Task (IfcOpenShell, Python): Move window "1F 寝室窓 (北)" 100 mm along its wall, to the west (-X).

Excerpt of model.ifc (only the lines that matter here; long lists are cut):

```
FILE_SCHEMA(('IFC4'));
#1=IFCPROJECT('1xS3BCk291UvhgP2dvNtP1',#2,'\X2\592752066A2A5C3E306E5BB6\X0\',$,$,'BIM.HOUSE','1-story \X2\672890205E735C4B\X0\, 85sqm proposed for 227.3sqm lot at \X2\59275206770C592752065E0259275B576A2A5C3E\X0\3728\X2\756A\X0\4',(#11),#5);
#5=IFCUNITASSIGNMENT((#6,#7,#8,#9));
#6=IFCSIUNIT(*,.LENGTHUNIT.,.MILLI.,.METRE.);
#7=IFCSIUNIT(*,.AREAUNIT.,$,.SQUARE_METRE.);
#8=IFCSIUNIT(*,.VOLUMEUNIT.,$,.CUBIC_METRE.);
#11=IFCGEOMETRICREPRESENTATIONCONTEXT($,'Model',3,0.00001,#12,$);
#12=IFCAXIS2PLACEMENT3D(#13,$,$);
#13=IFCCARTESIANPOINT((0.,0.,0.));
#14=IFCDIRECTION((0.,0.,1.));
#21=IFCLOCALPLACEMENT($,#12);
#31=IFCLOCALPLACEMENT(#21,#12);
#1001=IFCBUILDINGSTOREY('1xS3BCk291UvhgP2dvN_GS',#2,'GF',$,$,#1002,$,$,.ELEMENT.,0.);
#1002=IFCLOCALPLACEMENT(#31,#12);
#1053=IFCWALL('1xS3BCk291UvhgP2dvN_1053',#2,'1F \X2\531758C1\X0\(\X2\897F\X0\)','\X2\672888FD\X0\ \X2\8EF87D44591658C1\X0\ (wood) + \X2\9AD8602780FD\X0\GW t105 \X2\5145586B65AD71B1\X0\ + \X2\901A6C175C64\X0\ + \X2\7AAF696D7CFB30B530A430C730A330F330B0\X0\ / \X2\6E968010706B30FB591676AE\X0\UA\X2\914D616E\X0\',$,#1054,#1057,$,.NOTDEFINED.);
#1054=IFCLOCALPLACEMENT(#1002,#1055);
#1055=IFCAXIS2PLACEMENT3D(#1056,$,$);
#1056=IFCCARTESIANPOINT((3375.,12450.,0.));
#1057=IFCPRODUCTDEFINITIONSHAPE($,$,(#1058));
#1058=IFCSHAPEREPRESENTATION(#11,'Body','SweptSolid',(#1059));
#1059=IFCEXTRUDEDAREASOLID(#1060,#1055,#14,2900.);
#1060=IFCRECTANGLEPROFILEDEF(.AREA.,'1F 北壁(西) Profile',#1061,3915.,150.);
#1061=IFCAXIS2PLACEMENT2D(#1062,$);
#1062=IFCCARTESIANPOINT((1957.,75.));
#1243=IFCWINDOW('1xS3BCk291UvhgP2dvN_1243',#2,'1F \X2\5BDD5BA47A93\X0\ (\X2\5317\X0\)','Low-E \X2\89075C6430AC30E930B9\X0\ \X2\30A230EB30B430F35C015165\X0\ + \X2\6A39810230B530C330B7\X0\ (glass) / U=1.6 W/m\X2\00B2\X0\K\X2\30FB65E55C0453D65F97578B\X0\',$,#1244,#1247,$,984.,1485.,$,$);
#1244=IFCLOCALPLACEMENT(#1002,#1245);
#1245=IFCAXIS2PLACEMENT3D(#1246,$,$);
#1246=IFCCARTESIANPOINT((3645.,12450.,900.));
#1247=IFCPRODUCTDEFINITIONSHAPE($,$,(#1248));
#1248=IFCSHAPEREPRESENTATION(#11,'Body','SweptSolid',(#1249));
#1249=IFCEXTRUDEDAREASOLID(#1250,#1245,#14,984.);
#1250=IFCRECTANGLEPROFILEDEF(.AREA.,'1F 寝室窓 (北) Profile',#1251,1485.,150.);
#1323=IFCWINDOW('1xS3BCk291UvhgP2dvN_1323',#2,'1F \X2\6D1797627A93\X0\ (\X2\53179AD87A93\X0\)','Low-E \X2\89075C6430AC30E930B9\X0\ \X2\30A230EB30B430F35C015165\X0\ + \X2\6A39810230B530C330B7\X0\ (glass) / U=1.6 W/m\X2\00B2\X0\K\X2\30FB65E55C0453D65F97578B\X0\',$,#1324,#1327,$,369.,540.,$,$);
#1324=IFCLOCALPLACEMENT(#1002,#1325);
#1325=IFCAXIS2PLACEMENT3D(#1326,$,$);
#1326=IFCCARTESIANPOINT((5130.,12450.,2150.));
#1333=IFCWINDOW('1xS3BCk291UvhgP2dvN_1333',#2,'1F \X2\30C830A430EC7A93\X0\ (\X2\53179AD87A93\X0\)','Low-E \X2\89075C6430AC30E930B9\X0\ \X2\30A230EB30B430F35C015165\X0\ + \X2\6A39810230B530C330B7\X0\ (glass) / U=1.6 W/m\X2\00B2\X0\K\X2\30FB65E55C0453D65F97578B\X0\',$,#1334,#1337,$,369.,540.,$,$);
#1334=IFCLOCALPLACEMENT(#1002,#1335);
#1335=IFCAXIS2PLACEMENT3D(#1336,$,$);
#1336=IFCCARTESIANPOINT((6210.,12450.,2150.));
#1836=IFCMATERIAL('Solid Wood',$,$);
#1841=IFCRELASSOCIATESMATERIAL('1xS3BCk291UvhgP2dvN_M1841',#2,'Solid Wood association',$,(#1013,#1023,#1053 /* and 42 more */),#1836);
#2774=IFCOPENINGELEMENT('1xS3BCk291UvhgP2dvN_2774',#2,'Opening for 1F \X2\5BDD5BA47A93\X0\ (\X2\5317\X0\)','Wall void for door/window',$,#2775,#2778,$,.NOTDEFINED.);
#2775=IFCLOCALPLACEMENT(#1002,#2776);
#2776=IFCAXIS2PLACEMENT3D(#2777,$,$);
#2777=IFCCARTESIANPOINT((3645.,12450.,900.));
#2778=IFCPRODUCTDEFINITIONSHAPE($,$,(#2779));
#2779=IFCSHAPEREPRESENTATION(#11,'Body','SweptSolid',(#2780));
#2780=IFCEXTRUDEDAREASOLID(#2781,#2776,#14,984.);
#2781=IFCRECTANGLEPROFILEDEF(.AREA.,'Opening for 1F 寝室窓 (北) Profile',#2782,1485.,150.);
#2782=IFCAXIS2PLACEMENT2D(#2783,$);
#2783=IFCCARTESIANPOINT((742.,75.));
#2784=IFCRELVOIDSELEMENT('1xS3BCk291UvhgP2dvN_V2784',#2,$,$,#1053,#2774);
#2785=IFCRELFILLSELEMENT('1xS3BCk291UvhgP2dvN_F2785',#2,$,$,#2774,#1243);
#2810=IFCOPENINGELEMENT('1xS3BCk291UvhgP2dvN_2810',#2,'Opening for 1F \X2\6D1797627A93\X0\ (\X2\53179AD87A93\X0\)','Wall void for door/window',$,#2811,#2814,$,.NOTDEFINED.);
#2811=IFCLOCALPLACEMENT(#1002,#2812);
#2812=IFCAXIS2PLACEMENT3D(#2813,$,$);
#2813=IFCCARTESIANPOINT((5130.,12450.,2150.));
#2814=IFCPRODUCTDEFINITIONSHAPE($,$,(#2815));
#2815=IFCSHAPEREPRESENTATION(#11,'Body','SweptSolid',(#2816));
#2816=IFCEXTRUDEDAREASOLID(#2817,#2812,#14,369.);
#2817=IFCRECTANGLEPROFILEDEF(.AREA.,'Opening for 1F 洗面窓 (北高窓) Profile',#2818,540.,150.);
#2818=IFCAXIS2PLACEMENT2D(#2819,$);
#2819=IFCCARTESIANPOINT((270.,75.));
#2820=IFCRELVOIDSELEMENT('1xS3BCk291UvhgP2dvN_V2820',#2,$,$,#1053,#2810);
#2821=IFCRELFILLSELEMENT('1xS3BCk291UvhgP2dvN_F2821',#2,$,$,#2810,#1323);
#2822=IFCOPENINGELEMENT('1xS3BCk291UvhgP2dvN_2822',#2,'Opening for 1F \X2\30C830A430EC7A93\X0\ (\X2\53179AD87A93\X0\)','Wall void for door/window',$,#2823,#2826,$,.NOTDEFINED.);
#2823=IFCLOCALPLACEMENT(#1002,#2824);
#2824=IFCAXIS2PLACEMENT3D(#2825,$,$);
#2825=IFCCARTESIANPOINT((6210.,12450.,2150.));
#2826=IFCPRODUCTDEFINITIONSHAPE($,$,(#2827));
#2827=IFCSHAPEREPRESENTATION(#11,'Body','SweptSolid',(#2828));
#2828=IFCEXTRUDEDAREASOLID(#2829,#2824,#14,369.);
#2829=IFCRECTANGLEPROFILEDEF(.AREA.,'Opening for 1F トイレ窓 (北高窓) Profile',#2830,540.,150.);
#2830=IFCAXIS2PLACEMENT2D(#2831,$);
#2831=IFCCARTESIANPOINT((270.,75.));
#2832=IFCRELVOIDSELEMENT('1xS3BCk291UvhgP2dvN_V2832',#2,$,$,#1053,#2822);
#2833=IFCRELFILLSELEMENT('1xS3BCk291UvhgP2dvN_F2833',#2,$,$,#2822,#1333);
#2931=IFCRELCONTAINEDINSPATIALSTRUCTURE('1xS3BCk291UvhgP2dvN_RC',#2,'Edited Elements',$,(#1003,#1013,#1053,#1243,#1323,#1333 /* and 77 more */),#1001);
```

```python
import ifcopenshell
import ifcopenshell.api.geometry
import ifcopenshell.util.placement
import ifcopenshell.util.unit

model = ifcopenshell.open("model.ifc")
unit_scale = ifcopenshell.util.unit.calculate_unit_scale(model)

window = model.by_id(1243)
opening = window.FillsVoids[0].RelatingOpeningElement
wall = opening.VoidsElements[0].RelatingBuildingElement

wall_matrix = ifcopenshell.util.placement.get_local_placement(wall.ObjectPlacement)
shift = wall_matrix[:3, 0] * -0.1 / unit_scale
before = ifcopenshell.util.placement.get_local_placement(window.ObjectPlacement)[:3, 3].copy()

# The window is not placed relative to its opening, so move both.
for product in (opening, window):
    matrix = ifcopenshell.util.placement.get_local_placement(product.ObjectPlacement)
    matrix[:3, 3] += shift
    ifcopenshell.api.geometry.edit_object_placement(model, product=product, matrix=matrix, is_si=False)

after = ifcopenshell.util.placement.get_local_placement(window.ObjectPlacement)[:3, 3]
print("window moved by", (after - before).round(3) + 0.0)

model.write("model_edited.ifc")
```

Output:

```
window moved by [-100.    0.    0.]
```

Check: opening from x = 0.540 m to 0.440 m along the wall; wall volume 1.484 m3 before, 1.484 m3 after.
